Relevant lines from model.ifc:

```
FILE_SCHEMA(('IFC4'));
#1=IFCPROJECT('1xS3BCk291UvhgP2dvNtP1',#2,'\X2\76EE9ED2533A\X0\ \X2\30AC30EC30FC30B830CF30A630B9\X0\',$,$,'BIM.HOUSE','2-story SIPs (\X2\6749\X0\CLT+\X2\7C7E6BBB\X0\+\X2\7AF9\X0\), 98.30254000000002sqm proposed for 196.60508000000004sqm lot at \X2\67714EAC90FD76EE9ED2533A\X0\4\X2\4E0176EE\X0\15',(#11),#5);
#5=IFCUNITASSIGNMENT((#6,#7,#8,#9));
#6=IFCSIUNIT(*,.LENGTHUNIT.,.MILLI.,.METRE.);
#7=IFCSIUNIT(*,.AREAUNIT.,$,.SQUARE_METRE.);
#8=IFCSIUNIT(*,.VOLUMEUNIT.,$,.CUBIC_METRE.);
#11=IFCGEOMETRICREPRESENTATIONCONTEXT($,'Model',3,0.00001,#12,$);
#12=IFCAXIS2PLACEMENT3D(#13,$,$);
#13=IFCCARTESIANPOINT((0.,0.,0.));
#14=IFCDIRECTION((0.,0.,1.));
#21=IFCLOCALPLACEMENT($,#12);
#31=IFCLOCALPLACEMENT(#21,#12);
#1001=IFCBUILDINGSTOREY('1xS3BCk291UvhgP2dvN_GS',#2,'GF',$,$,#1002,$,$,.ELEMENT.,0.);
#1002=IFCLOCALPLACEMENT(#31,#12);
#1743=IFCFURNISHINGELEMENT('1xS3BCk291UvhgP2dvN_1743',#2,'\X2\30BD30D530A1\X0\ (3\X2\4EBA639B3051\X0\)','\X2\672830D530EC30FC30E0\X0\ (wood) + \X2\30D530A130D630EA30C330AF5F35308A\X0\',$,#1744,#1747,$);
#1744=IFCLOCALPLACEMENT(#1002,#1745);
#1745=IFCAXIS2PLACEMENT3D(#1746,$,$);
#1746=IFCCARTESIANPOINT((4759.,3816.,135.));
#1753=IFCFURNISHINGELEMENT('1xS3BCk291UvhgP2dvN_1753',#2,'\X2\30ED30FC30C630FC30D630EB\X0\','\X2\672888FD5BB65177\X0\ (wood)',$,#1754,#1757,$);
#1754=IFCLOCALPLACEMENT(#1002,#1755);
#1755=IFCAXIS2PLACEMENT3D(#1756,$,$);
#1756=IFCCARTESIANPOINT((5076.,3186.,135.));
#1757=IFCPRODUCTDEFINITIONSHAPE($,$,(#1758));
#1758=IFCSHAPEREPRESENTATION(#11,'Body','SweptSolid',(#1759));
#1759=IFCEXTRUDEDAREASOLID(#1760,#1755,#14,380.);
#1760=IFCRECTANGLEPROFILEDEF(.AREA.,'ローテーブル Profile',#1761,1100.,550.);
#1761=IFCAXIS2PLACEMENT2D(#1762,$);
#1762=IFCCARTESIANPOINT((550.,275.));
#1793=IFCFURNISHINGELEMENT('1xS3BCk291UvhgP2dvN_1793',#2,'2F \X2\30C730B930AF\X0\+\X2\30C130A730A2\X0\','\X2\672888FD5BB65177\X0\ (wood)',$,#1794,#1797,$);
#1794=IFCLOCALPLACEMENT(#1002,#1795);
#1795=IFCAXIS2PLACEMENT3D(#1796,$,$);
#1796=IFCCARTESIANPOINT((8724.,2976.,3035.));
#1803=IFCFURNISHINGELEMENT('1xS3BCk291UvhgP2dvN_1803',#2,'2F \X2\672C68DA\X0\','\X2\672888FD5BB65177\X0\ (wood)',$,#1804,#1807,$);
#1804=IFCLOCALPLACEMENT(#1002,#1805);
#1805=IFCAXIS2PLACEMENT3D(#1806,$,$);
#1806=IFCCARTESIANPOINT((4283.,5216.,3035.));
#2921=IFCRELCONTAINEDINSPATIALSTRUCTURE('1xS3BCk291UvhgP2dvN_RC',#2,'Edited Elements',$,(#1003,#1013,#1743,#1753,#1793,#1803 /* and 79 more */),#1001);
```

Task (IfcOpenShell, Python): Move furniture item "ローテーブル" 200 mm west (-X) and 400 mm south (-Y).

```python
import ifcopenshell
import ifcopenshell.api.geometry
import ifcopenshell.util.placement
import ifcopenshell.util.unit

model = ifcopenshell.open("model.ifc")
unit_scale = ifcopenshell.util.unit.calculate_unit_scale(model)

item = model.by_guid("1xS3BCk291UvhgP2dvN_1753")
matrix = ifcopenshell.util.placement.get_local_placement(item.ObjectPlacement)
matrix[0, 3] -= 0.2 / unit_scale
matrix[1, 3] -= 0.4 / unit_scale
ifcopenshell.api.geometry.edit_object_placement(model, product=item, matrix=matrix, is_si=False)

print(ifcopenshell.util.placement.get_local_placement(item.ObjectPlacement).round(3) + 0.0)

model.write("model-out.ifc")
```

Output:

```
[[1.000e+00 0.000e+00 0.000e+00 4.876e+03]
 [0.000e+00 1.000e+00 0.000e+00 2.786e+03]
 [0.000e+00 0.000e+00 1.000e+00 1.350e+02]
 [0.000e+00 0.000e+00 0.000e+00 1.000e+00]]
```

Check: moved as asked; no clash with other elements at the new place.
